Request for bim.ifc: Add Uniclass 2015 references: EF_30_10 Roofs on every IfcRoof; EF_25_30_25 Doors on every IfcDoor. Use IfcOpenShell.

First a look at what the model holds.

```python
import ifcopenshell

model = ifcopenshell.open("bim.ifc")
print(model.schema)
print("classifications:", [c.Name for c in model.by_type("IfcClassification")])
for ifc_class in ("IfcDoor", "IfcRoof", "IfcStair", "IfcWall", "IfcWindow"):
    print(ifc_class, len(model.by_type(ifc_class)))
```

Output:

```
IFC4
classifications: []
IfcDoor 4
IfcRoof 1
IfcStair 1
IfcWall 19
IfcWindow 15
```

```python
import ifcopenshell
import ifcopenshell.api.classification

model = ifcopenshell.open("bim.ifc")

system = ifcopenshell.api.classification.add_classification(model, classification="Uniclass 2015")

codes = {
    "IfcRoof": ("EF_30_10", "Roofs"),
    "IfcDoor": ("EF_25_30_25", "Doors"),
}
for ifc_class, (code, name) in codes.items():
    products = model.by_type(ifc_class)
    ifcopenshell.api.classification.add_reference(
        model, products=products, classification=system, identification=code, name=name
    )
    print(code, len(products))

model.write("bim-out.ifc")
```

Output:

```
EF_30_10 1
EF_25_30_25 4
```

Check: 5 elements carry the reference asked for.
